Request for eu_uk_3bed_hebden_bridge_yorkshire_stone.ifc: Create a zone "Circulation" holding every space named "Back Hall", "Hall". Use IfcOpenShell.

First a look at what the model holds.

```python
import ifcopenshell

model = ifcopenshell.open("eu_uk_3bed_hebden_bridge_yorkshire_stone.ifc")
print(model.schema)
seen = {}
for space in model.by_type("IfcSpace"):
    seen[space.LongName] = seen.get(space.LongName, 0) + 1
for name, count in sorted(seen.items(), key=str):
    print(count, "x", name)
print("zones:", [z.Name for z in model.by_type("IfcZone")][:20])
```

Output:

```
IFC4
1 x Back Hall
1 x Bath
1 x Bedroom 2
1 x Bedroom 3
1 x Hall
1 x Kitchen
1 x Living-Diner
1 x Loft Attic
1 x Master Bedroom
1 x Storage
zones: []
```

```python
import ifcopenshell
import ifcopenshell.api.group
import ifcopenshell.api.root

model = ifcopenshell.open("eu_uk_3bed_hebden_bridge_yorkshire_stone.ifc")

names = {"Back Hall", "Hall"}
spaces = [s for s in model.by_type("IfcSpace") if s.LongName in names]

zone = ifcopenshell.api.root.create_entity(model, ifc_class="IfcZone", name="Circulation")
ifcopenshell.api.group.assign_group(model, products=spaces, group=zone)
print(len(spaces), "spaces in", zone.Name)

model.write("eu_uk_3bed_hebden_bridge_yorkshire_stone-out.ifc")
```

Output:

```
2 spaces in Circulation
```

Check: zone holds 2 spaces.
